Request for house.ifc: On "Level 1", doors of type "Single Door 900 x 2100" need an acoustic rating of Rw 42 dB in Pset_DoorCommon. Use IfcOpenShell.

First a look at what the model holds.

```python
import ifcopenshell
import ifcopenshell.util.element

model = ifcopenshell.open("house.ifc")
print(model.schema)
storey = next(s for s in model.by_type("IfcBuildingStorey") if s.Name == "Level 1")
doors = [e for e in ifcopenshell.util.element.get_decomposition(storey) if e.is_a("IfcDoor")]
seen = {}
for e in doors:
    element_type = ifcopenshell.util.element.get_type(e)
    key = (element_type.Name if element_type != e and element_type else None, ifcopenshell.util.element.get_pset(e, "Pset_DoorCommon", "AcousticRating"))
    seen[key] = seen.get(key, 0) + 1
for (name, value), count in sorted(seen.items(), key=str):
    print(count, "x", name, "|", value)
```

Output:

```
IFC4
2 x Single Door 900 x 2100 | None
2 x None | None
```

```python
import ifcopenshell
import ifcopenshell.api.pset
import ifcopenshell.util.element

model = ifcopenshell.open("house.ifc")

storey = next(s for s in model.by_type("IfcBuildingStorey") if s.Name == "Level 1")
doors = [e for e in ifcopenshell.util.element.get_decomposition(storey) if e.is_a("IfcDoor")]

count = 0
for e in doors:
    element_type = ifcopenshell.util.element.get_type(e)
    if element_type in (None, e) or element_type.Name != "Single Door 900 x 2100":
        continue
    # add_pset returns the element's existing set when there is one.
    pset = ifcopenshell.api.pset.add_pset(model, product=e, name="Pset_DoorCommon")
    ifcopenshell.api.pset.edit_pset(model, pset=pset, properties={"AcousticRating": "Rw 42 dB"})
    count += 1

print(count, "doors updated")

model.write("house_updated.ifc")
```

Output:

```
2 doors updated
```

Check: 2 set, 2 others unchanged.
